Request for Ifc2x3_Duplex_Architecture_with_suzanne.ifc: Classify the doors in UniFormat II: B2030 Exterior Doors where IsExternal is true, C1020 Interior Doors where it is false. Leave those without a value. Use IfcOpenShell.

First a look at what the model holds.

```python
import ifcopenshell
import ifcopenshell.util.element

model = ifcopenshell.open("Ifc2x3_Duplex_Architecture_with_suzanne.ifc")
print(model.schema)
print("classifications:", [c.Name for c in model.by_type("IfcClassification")])
values = [ifcopenshell.util.element.get_pset(e, "Pset_DoorCommon", "IsExternal") for e in model.by_type("IfcDoor")]
for value in (True, False, None):
    print("IsExternal", value, values.count(value))
```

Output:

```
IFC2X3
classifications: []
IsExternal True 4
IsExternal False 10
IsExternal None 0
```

```python
import ifcopenshell
import ifcopenshell.api.classification
import ifcopenshell.util.element

model = ifcopenshell.open("Ifc2x3_Duplex_Architecture_with_suzanne.ifc")

# IFC2X3 requires Source and Edition and has no link from the project to the system.
system = model.create_entity("IfcClassification", Source="ASTM", Edition="E1557", Name="UniFormat II")

doors = model.by_type("IfcDoor")
external = {e: ifcopenshell.util.element.get_pset(e, "Pset_DoorCommon", "IsExternal") for e in doors}
for flag, code, name in ((True, "B2030", "Exterior Doors"), (False, "C1020", "Interior Doors")):
    products = [e for e in doors if external[e] is flag]
    ifcopenshell.api.classification.add_reference(
        model, products=products, classification=system, identification=code, name=name
    )
    print(code, len(products))

model.write("Ifc2x3_Duplex_Architecture_with_suzanne_edited.ifc")
```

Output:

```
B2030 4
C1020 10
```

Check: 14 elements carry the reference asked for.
